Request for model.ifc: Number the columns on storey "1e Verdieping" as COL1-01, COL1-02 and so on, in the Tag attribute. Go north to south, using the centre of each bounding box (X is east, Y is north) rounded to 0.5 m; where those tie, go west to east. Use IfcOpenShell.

First a look at what the model holds.

```python
import ifcopenshell
import ifcopenshell.util.element
import ifcopenshell.util.placement

model = ifcopenshell.open("model.ifc")
print(model.schema)
storey = next(s for s in model.by_type("IfcBuildingStorey") if s.Name == "1e Verdieping")
columns = [e for e in ifcopenshell.util.element.get_decomposition(storey) if e.is_a("IfcColumn")]
for e in sorted(columns, key=lambda e: e.id()):
    origin = ifcopenshell.util.placement.get_local_placement(e.ObjectPlacement)[:3, 3]
    print(e.id(), e.Tag, e.Name, origin.round(2) + 0.0, sep=" | ")
```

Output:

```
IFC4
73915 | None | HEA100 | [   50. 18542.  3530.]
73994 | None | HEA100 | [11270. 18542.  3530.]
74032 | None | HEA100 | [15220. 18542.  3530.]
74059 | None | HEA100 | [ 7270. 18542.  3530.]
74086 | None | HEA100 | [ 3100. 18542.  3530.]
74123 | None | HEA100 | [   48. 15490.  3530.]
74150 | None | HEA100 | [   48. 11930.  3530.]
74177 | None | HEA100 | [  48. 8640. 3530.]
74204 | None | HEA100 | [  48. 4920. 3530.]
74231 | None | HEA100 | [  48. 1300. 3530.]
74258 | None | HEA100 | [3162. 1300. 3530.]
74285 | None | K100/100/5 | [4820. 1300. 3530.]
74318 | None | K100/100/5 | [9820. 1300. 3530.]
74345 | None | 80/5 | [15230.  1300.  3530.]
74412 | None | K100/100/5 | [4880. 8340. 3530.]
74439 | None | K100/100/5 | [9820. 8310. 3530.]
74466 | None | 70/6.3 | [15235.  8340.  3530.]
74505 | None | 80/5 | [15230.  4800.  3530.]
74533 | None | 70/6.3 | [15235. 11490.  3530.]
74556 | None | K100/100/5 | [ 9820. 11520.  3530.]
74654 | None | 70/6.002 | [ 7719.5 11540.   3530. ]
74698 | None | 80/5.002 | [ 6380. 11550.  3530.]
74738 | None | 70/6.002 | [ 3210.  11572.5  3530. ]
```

```python
import ifcopenshell
import ifcopenshell.geom
import ifcopenshell.util.element
import ifcopenshell.util.shape

model = ifcopenshell.open("model.ifc")
settings = ifcopenshell.geom.settings()
settings.set("use-world-coords", True)


def centre(element):
    shape = ifcopenshell.geom.create_shape(settings, element)
    return ifcopenshell.util.shape.get_bbox_centroid(shape.geometry)


storey = next(s for s in model.by_type("IfcBuildingStorey") if s.Name == "1e Verdieping")
columns = [e for e in ifcopenshell.util.element.get_decomposition(storey) if e.is_a("IfcColumn")]

# Insertion points can sit at a corner or the storey origin, so sort by the geometry (in metres).
centres = {e: centre(e) for e in columns}
columns.sort(key=lambda e: (-round(centres[e][1] / 0.5), centres[e][0]))

for i, e in enumerate(columns, start=1):
    number = f"COL1-{i:02d}"
    e.Tag = number
    print(e.id(), number)

model.write("model_rev.ifc")
```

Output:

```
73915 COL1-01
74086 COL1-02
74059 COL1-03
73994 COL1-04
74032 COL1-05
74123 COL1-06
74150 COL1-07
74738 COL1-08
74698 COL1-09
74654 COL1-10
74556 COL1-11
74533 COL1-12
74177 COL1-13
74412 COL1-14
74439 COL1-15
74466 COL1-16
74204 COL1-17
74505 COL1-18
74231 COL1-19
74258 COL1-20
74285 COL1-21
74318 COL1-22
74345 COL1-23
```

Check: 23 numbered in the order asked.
